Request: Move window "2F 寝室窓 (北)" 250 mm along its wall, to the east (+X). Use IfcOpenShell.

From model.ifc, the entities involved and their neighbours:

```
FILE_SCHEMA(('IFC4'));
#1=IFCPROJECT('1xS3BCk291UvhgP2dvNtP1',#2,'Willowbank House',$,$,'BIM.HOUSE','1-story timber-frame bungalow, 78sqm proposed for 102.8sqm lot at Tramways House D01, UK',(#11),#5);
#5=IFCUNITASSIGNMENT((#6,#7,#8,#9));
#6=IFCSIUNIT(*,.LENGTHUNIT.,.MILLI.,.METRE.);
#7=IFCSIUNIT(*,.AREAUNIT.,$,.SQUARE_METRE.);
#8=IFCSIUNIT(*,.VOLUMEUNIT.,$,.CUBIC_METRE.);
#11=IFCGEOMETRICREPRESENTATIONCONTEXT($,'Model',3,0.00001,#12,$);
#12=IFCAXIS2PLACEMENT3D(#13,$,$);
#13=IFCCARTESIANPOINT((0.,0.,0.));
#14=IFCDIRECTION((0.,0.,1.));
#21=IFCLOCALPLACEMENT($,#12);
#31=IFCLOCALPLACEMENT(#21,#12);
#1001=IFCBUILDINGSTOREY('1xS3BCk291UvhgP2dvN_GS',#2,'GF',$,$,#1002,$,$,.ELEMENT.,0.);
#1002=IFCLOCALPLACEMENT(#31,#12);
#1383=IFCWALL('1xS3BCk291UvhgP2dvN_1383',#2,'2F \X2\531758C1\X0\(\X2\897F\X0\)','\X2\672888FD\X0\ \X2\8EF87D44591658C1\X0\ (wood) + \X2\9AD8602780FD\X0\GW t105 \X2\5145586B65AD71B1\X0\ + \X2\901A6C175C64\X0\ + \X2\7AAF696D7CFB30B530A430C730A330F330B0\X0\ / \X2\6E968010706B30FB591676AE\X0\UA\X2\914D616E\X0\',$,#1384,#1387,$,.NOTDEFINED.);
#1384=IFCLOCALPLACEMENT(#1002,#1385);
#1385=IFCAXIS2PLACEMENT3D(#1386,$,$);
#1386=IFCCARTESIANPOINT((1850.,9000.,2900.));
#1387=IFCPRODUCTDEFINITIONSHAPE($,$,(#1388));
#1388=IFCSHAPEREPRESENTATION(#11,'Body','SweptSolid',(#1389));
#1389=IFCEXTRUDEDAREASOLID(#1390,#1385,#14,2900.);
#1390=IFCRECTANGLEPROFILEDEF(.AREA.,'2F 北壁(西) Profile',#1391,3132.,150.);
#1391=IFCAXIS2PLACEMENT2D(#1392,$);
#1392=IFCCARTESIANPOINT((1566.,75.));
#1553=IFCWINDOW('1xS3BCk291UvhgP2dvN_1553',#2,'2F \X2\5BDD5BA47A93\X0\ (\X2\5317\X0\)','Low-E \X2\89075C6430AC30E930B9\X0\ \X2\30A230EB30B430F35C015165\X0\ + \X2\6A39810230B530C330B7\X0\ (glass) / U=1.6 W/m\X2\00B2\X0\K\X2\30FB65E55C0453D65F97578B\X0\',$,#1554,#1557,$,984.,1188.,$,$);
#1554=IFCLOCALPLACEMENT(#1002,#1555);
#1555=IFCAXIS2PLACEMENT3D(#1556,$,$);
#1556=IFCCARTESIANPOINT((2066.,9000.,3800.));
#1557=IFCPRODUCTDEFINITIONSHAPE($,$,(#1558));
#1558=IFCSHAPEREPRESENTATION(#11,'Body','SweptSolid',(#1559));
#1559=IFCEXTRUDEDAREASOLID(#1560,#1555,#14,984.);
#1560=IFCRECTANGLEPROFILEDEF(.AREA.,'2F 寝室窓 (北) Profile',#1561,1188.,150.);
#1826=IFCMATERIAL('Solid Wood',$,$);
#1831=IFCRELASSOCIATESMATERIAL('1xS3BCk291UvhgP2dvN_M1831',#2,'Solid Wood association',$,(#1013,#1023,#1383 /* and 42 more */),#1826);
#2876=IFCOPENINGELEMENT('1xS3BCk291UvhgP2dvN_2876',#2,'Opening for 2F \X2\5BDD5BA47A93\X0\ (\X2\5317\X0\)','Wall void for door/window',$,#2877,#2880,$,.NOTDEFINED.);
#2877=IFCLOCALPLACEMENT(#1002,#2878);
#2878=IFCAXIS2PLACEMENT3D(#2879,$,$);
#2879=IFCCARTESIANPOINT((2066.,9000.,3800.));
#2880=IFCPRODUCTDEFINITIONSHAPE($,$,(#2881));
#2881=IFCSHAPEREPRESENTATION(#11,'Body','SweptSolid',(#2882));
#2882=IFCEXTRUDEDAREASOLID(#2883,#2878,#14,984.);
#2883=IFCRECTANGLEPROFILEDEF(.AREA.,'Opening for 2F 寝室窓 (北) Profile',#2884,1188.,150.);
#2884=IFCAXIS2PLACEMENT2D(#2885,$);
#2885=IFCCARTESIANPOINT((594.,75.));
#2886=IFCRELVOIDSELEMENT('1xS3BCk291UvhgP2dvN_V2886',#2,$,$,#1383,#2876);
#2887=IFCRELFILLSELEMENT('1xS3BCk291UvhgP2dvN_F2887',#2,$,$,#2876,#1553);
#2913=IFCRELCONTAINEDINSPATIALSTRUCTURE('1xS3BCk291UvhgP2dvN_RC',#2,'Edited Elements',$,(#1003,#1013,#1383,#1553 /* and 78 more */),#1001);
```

```python
import ifcopenshell
import ifcopenshell.api.geometry
import ifcopenshell.util.placement
import ifcopenshell.util.unit

model = ifcopenshell.open("model.ifc")
unit_scale = ifcopenshell.util.unit.calculate_unit_scale(model)

window = model.by_guid("1xS3BCk291UvhgP2dvN_1553")
opening = window.FillsVoids[0].RelatingOpeningElement
wall = opening.VoidsElements[0].RelatingBuildingElement

wall_matrix = ifcopenshell.util.placement.get_local_placement(wall.ObjectPlacement)
shift = wall_matrix[:3, 0] * 0.25 / unit_scale
before = ifcopenshell.util.placement.get_local_placement(window.ObjectPlacement)[:3, 3].copy()

# The window is not placed relative to its opening, so move both.
for product in (opening, window):
    matrix = ifcopenshell.util.placement.get_local_placement(product.ObjectPlacement)
    matrix[:3, 3] += shift
    ifcopenshell.api.geometry.edit_object_placement(model, product=product, matrix=matrix, is_si=False)

after = ifcopenshell.util.placement.get_local_placement(window.ObjectPlacement)[:3, 3]
print("window moved by", (after - before).round(3) + 0.0)

model.write("model_rev.ifc")
```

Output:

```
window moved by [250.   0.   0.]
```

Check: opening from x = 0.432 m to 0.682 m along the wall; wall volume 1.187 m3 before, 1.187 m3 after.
